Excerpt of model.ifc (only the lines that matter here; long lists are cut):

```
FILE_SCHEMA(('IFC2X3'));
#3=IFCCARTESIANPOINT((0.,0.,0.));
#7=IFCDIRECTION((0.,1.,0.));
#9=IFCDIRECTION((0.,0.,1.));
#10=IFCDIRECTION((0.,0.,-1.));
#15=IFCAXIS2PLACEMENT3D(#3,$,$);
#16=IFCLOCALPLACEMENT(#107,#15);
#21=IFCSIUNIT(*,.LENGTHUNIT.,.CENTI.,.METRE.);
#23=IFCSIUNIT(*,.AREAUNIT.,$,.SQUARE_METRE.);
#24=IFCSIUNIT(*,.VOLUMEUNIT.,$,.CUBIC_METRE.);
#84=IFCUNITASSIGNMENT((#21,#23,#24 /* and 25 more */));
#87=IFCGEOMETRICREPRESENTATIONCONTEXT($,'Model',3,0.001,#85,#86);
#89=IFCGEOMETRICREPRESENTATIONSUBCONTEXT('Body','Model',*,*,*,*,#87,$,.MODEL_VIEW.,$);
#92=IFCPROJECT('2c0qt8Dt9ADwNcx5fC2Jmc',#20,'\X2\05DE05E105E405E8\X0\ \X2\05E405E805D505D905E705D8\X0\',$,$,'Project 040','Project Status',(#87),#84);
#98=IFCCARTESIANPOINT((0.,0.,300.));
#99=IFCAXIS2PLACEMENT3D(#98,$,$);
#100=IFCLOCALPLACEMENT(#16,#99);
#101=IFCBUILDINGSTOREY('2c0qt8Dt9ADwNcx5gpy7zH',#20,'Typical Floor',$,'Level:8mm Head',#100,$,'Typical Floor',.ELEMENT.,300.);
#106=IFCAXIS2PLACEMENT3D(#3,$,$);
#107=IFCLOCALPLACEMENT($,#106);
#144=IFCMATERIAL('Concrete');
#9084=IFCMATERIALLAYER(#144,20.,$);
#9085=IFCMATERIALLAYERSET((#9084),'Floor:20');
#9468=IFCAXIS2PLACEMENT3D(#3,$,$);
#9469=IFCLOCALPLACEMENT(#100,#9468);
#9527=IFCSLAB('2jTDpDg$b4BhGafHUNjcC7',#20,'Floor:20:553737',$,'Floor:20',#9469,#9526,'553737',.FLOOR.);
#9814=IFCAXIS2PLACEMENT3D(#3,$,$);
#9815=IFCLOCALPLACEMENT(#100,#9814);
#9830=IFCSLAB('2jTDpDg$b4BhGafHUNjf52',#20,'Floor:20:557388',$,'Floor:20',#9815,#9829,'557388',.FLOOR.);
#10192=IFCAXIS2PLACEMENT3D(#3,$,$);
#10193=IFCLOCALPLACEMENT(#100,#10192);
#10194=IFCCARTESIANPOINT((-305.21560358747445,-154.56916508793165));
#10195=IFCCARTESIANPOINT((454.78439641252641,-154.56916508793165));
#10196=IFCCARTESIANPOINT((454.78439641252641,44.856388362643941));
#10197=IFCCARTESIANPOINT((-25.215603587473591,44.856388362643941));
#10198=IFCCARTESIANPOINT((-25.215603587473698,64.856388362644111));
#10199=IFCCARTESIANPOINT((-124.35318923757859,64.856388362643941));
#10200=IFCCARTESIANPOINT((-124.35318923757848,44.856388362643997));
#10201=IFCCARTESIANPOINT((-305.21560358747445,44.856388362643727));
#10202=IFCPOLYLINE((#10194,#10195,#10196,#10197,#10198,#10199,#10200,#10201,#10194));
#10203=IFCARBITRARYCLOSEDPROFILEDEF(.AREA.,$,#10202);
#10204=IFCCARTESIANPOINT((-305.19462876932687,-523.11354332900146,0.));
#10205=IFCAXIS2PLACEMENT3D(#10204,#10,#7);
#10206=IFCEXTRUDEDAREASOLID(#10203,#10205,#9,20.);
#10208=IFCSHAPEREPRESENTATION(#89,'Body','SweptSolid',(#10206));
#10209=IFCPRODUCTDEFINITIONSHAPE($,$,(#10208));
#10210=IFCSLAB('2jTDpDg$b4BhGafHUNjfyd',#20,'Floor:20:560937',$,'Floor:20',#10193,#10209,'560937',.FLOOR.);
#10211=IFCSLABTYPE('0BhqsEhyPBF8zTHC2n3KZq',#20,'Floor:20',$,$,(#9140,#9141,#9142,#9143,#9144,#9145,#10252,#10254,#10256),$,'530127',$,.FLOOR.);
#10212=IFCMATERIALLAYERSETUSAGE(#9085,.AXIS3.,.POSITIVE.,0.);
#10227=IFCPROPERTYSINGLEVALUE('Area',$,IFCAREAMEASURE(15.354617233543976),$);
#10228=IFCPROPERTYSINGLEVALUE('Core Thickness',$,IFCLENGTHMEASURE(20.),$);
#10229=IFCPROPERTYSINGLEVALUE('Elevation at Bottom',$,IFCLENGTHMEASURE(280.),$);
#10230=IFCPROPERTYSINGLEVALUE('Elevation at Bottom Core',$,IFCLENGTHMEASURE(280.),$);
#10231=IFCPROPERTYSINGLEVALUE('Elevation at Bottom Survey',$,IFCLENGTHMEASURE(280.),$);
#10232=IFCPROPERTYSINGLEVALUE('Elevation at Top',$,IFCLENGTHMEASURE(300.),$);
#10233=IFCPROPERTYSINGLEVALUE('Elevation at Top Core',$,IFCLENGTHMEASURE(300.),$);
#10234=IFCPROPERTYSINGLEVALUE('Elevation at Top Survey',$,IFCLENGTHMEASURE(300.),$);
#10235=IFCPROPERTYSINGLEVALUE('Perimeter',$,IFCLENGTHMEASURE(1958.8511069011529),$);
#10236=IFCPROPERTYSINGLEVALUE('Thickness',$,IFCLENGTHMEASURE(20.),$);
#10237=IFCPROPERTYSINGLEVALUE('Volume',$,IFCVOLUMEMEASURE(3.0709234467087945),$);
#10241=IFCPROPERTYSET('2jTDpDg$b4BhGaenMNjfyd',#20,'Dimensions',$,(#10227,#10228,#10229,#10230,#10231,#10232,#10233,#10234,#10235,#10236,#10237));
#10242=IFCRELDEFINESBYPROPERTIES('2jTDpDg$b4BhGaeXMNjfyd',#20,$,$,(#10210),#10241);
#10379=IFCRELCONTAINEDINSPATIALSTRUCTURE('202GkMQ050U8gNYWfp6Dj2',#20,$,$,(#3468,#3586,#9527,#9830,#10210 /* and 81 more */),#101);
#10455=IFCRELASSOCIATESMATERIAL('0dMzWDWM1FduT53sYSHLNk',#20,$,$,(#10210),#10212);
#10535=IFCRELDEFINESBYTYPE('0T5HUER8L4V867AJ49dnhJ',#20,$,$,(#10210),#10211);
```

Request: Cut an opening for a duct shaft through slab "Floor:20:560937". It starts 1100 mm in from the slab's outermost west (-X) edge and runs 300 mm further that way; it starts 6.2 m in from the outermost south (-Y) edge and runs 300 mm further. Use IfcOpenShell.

```python
import numpy as np
import ifcopenshell
import ifcopenshell.api.feature
import ifcopenshell.api.geometry
import ifcopenshell.api.pset
import ifcopenshell.api.root
import ifcopenshell.geom
import ifcopenshell.util.element
import ifcopenshell.util.placement
import ifcopenshell.util.representation
import ifcopenshell.util.shape
import ifcopenshell.util.unit

model = ifcopenshell.open("model.ifc")
unit_scale = ifcopenshell.util.unit.calculate_unit_scale(model)
area_scale = ifcopenshell.util.unit.calculate_unit_scale(model, "AREAUNIT")
volume_scale = ifcopenshell.util.unit.calculate_unit_scale(model, "VOLUMEUNIT")
settings = ifcopenshell.geom.settings()


def volume(element):
    """Net volume in cubic metres, openings subtracted."""
    shape = ifcopenshell.geom.create_shape(settings, element)
    return ifcopenshell.util.shape.get_volume(shape.geometry)


slab = model.by_guid("2jTDpDg$b4BhGafHUNjfyd")
before = volume(slab)

# Extent in the slab's own axes, in metres. The edges named are its -X and -Y sides.
slab_shape = ifcopenshell.geom.create_shape(settings, slab)
vertices = ifcopenshell.util.shape.get_vertices(slab_shape.geometry)
x_min, y_min, bottom = vertices.min(axis=0)
top = vertices[:, 2].max()

opening = ifcopenshell.api.root.create_entity(model, ifc_class="IfcOpeningElement", name="Duct shaft opening")
context = ifcopenshell.util.representation.get_context(model, "Model", "Body", "MODEL_VIEW")
width, depth = 0.3, 0.3
outline = [(0.0, 0.0), (width, 0.0), (width, depth), (0.0, depth), (0.0, 0.0)]
# Overshoot both faces by 50 mm so the cut is clean.
shape = ifcopenshell.api.geometry.add_slab_representation(
    model, context=context, depth=top - bottom + 0.1, polyline=outline
)
ifcopenshell.api.geometry.assign_representation(model, product=opening, representation=shape)

matrix = ifcopenshell.util.placement.get_local_placement(slab.ObjectPlacement)
matrix[:, 3] = matrix @ np.append(np.array([x_min + 1.1, y_min + 6.2, bottom - 0.05]) / unit_scale, 1.0)
ifcopenshell.api.geometry.edit_object_placement(model, product=opening, matrix=matrix, is_si=False)
ifcopenshell.api.feature.add_feature(model, feature=opening, element=slab)

after = volume(slab)

# Update the slab's stored quantities.
pset = model.by_id(ifcopenshell.util.element.get_pset(slab, "Dimensions", should_inherit=False)["id"])
ifcopenshell.api.pset.edit_pset(model, pset=pset, properties={
    "Area": model.create_entity("IfcAreaMeasure", after / (top - bottom) / area_scale),
    "Volume": model.create_entity("IfcVolumeMeasure", after / volume_scale),
})

print(f"slab volume {before:.3f} -> {after:.3f} m3")

model.write("model-out.ifc")
```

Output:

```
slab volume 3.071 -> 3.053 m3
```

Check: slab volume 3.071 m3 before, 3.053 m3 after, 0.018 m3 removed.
